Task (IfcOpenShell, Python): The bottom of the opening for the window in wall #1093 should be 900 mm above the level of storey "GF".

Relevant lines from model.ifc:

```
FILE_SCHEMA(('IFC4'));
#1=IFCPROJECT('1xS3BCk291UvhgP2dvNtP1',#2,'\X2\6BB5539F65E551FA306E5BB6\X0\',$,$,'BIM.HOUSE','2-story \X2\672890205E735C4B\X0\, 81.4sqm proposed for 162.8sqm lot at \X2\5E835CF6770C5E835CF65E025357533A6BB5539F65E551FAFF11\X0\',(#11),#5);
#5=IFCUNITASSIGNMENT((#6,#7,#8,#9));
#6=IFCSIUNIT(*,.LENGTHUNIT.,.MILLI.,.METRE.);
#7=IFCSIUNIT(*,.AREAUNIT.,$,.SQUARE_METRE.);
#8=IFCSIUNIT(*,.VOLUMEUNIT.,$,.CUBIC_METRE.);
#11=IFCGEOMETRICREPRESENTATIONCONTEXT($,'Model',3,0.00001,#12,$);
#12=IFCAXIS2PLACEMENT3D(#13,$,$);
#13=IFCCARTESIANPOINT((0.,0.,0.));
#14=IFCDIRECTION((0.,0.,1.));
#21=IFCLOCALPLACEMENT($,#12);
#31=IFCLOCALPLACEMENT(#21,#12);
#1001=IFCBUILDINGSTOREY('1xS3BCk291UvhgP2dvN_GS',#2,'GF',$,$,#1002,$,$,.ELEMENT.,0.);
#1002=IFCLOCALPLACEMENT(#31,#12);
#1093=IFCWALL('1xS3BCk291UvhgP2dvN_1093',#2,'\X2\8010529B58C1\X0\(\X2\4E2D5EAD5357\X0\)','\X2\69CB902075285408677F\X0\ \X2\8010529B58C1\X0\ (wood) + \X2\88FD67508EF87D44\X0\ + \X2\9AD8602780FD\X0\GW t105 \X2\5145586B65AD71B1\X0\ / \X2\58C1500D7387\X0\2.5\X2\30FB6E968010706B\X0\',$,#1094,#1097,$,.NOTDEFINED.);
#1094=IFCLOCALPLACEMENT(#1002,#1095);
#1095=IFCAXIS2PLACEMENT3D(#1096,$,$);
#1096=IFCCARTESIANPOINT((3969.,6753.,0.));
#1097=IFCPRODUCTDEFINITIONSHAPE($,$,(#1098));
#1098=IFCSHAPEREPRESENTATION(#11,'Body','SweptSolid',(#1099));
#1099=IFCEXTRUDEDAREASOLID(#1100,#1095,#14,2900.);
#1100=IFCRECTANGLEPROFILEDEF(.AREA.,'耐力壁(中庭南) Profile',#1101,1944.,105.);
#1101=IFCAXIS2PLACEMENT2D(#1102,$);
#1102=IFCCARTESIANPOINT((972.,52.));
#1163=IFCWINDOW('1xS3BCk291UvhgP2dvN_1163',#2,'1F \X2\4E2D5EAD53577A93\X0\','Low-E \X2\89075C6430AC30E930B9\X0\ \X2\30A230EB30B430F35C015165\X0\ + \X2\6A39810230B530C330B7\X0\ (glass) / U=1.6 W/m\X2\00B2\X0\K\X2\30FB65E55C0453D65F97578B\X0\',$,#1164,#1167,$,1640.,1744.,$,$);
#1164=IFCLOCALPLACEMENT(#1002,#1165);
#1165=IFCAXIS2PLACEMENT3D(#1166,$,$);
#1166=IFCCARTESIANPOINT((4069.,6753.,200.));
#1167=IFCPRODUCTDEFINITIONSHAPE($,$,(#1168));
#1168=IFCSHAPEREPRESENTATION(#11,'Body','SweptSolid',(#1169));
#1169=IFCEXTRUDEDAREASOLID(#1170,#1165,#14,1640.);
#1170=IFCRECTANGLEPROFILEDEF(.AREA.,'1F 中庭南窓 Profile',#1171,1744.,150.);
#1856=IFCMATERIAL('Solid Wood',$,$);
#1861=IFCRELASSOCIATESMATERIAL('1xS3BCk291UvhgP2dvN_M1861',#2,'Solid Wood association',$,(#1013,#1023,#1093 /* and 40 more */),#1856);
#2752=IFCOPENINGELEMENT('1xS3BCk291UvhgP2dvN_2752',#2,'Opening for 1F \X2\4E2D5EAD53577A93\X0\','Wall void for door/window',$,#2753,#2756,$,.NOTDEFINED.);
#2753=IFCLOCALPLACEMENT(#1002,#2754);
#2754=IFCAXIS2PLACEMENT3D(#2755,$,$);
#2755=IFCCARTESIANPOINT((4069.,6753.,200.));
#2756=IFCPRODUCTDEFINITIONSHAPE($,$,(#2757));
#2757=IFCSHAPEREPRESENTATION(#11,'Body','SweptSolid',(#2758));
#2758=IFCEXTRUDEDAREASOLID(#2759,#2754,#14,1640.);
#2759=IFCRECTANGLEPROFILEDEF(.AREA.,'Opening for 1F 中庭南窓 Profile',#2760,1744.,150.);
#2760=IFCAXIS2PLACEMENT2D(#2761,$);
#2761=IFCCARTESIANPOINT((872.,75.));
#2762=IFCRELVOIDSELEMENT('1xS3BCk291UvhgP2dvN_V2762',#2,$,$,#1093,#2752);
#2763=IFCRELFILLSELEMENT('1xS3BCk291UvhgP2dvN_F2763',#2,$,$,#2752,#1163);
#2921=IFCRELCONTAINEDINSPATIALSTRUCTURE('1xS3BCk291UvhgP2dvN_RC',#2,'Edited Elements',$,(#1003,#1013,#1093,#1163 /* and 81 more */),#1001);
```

```python
import numpy as np
import ifcopenshell
import ifcopenshell.api.geometry
import ifcopenshell.geom
import ifcopenshell.util.element
import ifcopenshell.util.placement
import ifcopenshell.util.shape
import ifcopenshell.util.unit

model = ifcopenshell.open("model.ifc")
unit_scale = ifcopenshell.util.unit.calculate_unit_scale(model)

window = model.by_guid("1xS3BCk291UvhgP2dvN_1163")
opening = window.FillsVoids[0].RelatingOpeningElement
storey = ifcopenshell.util.element.get_container(window, ifc_class="IfcBuildingStorey")
level = ifcopenshell.util.placement.get_local_placement(storey.ObjectPlacement)[2, 3]

# The opening's origin need not be at the sill, so measure its lowest point.
shape = ifcopenshell.geom.create_shape(ifcopenshell.geom.settings(), opening)
bottom = ifcopenshell.util.shape.get_shape_bottom_elevation(shape, shape.geometry) / unit_scale
dz = level + 900.0 - bottom

shift = np.array([0.0, 0.0, dz])
# The window is not placed relative to its opening, so move both.
for product in (opening, window):
    matrix = ifcopenshell.util.placement.get_local_placement(product.ObjectPlacement)
    matrix[:3, 3] += shift
    ifcopenshell.api.geometry.edit_object_placement(model, product=product, matrix=matrix, is_si=False)

print(f"moved by {dz * unit_scale:+.3f} m")

model.write("model_edited.ifc")
```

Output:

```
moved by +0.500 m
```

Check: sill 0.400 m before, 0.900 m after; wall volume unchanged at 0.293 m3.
